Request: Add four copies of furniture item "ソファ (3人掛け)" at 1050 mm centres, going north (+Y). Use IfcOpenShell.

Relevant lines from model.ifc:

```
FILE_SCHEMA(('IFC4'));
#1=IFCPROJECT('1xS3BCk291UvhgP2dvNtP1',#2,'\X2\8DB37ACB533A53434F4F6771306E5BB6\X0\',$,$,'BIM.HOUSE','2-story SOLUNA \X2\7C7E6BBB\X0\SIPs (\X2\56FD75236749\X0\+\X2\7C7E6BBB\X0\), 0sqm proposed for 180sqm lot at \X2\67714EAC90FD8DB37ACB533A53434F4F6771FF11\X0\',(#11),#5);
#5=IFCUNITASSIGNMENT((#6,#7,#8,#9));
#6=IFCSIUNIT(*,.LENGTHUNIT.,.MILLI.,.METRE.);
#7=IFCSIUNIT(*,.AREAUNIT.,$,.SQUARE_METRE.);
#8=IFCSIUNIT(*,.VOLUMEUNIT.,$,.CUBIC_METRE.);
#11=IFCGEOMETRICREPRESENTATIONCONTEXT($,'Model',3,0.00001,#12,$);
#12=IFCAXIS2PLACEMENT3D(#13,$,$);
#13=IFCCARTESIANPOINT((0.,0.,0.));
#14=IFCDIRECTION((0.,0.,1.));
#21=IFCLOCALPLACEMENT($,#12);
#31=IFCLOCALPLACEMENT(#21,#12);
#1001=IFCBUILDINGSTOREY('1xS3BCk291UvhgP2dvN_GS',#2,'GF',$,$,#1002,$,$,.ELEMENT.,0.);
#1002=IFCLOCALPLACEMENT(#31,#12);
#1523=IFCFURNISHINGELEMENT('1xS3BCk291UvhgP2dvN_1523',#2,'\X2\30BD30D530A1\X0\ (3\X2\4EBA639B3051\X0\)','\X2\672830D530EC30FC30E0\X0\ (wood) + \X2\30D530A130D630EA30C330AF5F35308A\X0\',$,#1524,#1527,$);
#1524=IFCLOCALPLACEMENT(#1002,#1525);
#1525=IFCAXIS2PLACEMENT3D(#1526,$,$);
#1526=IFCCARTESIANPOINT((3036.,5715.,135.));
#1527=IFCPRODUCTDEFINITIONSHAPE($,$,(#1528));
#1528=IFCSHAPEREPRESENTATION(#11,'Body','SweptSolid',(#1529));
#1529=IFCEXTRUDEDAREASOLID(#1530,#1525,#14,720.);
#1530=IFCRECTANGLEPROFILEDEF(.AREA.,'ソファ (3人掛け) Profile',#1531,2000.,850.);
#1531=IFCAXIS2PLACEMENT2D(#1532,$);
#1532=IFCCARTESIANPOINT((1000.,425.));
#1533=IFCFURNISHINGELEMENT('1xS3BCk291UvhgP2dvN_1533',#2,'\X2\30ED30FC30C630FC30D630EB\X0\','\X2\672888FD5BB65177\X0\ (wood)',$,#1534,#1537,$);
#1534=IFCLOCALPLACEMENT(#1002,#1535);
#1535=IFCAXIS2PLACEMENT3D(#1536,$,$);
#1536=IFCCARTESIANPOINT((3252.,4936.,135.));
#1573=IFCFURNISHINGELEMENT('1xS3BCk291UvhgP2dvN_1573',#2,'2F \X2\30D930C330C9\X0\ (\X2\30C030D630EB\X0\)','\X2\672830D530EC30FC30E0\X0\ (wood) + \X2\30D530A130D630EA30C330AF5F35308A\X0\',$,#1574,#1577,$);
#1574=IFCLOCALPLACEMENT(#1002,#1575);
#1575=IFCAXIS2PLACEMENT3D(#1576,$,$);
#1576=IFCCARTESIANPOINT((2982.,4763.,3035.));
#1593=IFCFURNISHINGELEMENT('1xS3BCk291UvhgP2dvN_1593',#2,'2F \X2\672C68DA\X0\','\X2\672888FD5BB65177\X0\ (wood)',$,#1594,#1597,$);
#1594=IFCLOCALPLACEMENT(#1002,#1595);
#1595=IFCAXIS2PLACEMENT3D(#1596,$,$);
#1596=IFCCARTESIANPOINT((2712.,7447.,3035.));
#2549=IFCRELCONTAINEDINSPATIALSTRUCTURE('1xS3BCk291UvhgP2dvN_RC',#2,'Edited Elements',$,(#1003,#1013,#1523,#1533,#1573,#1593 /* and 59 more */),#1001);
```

```python
import numpy as np
import ifcopenshell
import ifcopenshell.api.geometry
import ifcopenshell.api.root
import ifcopenshell.util.element
import ifcopenshell.util.placement

model = ifcopenshell.open("model.ifc")


def reuse_history(source, copy):
    """copy_class also copies each property set's owner history, people and application; keep the originals."""
    for rel in copy.IsDefinedBy:
        if rel.is_a("IfcRelDefinesByProperties") and (history := rel.RelatingPropertyDefinition.OwnerHistory):
            rel.RelatingPropertyDefinition.OwnerHistory = source.OwnerHistory
            ifcopenshell.util.element.remove_deep2(model, history)


source = model.by_guid("1xS3BCk291UvhgP2dvN_1523")
base = ifcopenshell.util.placement.get_local_placement(source.ObjectPlacement)
step = np.array([0.0, 1.0, 0.0]) * 1050.0

for i in range(1, 5):
    copy = ifcopenshell.api.root.copy_class(model, product=source)
    copy.Representation = ifcopenshell.util.element.copy_deep(
        model, source.Representation, exclude=["IfcGeometricRepresentationContext", "IfcRepresentationMap"]
    )
    reuse_history(source, copy)
    matrix = base.copy()
    matrix[:3, 3] += i * step
    print("added at", matrix[:3, 3].round(3) + 0.0)
    ifcopenshell.api.geometry.edit_object_placement(model, product=copy, matrix=matrix, is_si=False)

model.write("model_edited.ifc")
```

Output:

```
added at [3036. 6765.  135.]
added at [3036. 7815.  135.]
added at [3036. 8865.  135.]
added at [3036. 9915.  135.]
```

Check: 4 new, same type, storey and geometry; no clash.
